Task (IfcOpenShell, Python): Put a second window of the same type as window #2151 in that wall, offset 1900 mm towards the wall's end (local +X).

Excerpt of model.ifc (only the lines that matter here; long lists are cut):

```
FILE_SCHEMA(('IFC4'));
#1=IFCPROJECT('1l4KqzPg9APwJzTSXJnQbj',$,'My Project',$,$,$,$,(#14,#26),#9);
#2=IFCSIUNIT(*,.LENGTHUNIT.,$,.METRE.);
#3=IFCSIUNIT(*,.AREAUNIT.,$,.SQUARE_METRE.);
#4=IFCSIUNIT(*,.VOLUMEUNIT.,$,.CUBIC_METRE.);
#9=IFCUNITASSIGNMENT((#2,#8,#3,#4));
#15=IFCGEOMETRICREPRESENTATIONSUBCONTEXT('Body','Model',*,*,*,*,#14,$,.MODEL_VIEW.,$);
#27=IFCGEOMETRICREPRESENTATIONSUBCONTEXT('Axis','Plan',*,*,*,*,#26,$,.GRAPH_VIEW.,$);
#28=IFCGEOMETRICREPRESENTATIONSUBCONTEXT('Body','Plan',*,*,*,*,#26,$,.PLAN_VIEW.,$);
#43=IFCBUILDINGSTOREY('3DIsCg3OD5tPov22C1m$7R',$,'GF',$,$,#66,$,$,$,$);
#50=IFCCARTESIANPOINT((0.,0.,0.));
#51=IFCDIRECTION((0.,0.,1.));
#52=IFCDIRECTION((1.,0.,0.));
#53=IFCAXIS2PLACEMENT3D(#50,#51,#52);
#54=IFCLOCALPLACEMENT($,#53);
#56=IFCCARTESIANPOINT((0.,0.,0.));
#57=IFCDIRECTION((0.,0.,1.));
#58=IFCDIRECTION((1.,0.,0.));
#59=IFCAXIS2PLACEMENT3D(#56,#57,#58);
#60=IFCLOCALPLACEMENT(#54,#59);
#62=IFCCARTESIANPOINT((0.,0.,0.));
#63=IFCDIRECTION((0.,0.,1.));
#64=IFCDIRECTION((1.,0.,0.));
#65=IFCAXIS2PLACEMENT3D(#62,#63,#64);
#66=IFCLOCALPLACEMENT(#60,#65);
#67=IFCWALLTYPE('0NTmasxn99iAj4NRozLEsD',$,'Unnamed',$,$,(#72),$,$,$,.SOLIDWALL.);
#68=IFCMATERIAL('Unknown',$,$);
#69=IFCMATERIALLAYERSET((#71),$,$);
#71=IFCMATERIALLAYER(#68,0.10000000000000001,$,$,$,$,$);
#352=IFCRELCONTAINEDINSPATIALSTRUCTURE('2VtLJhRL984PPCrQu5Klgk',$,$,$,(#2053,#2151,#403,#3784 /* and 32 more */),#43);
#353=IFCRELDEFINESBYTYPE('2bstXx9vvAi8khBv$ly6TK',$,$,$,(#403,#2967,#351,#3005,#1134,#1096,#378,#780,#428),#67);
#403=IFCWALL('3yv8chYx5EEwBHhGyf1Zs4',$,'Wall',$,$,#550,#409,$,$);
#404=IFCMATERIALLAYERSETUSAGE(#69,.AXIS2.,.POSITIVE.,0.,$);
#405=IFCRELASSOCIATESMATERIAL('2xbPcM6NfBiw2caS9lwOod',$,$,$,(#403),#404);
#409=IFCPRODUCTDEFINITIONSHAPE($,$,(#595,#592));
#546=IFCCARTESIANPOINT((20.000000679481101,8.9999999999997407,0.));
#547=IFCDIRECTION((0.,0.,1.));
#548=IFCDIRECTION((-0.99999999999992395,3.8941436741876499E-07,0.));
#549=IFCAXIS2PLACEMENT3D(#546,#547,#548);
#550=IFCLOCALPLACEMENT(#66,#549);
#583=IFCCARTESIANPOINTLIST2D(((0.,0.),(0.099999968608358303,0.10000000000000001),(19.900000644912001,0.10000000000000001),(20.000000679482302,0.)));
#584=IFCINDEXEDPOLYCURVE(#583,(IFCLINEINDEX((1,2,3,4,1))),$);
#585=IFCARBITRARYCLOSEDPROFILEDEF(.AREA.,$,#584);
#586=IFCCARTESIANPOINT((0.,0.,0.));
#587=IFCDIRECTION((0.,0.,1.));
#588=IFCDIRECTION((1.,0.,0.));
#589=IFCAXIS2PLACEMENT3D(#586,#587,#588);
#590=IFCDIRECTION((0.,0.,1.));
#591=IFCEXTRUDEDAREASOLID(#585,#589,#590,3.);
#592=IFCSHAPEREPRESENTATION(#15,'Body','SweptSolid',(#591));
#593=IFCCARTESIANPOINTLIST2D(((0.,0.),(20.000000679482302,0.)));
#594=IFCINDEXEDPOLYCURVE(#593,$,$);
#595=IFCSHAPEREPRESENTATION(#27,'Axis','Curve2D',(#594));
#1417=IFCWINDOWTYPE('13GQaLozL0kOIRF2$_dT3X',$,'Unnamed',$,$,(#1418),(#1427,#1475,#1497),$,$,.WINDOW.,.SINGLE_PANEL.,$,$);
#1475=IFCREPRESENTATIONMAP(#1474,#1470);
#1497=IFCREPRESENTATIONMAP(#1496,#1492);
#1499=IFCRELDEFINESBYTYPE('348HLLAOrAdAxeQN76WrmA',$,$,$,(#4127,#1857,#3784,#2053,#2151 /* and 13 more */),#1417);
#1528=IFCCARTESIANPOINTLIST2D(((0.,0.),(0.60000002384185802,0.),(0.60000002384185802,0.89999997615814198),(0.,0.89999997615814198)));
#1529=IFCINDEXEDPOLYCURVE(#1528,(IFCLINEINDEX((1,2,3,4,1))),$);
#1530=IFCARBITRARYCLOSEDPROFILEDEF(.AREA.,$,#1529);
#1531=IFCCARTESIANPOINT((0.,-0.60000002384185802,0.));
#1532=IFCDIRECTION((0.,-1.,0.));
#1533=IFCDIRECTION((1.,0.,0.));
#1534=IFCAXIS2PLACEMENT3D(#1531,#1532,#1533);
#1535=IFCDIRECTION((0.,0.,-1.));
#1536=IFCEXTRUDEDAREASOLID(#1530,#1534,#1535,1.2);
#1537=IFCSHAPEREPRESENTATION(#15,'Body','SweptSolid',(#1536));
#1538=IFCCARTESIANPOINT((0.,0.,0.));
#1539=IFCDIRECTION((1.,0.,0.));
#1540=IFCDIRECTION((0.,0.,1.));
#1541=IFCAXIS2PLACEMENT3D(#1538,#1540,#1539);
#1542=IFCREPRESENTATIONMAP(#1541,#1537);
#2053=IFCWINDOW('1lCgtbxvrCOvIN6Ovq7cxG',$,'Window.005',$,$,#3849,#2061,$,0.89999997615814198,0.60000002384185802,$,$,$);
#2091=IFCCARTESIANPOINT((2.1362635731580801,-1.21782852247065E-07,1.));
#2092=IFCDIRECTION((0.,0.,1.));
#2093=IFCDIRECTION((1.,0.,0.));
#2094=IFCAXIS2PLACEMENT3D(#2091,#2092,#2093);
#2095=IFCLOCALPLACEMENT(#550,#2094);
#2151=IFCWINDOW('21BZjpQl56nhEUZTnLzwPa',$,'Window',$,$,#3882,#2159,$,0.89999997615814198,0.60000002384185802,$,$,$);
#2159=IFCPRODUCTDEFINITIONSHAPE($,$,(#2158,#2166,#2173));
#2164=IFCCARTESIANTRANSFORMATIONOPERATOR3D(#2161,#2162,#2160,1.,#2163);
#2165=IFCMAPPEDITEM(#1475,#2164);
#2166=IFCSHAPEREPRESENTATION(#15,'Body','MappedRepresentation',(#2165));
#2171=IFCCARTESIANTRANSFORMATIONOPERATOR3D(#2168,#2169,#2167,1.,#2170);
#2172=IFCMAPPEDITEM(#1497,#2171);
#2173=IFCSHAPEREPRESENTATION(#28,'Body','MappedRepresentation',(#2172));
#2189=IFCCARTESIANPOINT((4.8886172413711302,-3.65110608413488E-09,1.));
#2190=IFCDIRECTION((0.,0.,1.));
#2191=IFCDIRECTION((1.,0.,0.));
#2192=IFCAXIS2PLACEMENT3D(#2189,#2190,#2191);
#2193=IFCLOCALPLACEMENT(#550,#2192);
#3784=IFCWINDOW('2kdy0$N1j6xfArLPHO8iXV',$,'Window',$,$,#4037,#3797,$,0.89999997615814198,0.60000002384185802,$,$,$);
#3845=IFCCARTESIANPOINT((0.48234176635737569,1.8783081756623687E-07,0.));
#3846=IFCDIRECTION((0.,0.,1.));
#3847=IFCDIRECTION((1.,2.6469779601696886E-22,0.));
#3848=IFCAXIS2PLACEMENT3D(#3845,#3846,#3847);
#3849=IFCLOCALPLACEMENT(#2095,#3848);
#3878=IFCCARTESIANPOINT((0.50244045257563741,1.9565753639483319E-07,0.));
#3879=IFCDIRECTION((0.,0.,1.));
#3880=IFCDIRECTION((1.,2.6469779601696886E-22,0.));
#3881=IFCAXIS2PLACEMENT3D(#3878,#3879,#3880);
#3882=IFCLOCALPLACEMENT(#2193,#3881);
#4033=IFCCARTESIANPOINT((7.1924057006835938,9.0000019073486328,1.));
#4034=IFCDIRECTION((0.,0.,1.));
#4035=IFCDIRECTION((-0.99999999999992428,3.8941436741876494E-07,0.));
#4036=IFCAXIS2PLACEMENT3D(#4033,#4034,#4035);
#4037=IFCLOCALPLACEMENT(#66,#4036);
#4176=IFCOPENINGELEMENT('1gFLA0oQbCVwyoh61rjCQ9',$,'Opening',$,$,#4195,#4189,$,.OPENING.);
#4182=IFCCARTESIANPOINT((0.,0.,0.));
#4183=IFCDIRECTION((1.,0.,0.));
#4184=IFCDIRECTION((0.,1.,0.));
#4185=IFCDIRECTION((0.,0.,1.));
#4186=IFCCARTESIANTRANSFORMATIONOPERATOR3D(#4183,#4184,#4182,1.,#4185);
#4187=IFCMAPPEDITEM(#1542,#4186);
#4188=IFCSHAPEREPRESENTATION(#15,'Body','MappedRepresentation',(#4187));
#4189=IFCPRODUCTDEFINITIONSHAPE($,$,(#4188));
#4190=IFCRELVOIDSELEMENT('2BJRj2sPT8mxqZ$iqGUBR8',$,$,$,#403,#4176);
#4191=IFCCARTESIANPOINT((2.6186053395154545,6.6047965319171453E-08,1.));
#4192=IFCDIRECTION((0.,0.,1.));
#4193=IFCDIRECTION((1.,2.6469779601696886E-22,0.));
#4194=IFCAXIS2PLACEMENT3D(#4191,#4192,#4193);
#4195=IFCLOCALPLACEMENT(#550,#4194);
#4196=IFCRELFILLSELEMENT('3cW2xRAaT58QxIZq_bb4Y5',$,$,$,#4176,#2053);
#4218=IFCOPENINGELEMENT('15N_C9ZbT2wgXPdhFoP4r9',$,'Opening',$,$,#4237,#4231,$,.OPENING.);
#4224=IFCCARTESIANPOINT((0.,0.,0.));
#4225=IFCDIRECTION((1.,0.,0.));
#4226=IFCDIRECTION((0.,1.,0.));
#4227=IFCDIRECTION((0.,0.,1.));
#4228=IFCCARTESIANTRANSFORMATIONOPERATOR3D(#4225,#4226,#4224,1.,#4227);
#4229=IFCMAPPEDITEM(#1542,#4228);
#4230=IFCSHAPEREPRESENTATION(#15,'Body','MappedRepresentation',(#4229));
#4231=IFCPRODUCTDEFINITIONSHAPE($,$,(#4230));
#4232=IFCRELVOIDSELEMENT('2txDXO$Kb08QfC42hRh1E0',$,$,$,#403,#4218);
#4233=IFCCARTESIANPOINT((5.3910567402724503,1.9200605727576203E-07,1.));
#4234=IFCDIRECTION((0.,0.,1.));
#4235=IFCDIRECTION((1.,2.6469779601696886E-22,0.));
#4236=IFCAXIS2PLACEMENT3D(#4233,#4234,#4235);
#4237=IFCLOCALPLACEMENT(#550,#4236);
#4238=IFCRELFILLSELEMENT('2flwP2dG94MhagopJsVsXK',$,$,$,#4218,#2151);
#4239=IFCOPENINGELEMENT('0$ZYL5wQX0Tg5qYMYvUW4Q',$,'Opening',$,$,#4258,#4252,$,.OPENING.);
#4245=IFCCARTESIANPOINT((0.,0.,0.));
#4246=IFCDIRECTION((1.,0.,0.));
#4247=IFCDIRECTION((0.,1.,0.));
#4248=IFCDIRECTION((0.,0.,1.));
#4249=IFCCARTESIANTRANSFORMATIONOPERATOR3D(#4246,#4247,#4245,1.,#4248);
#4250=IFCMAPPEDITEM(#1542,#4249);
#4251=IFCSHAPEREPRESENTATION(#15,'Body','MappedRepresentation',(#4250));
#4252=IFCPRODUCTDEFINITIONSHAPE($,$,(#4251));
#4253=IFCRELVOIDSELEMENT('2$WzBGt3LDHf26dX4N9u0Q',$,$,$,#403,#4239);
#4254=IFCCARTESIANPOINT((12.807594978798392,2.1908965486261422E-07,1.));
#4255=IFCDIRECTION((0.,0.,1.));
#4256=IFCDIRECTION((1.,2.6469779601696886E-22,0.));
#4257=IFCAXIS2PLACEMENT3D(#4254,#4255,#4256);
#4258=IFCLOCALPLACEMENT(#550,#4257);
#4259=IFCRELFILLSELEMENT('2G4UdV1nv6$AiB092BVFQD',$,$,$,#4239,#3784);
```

```python
import ifcopenshell
import ifcopenshell.api.feature
import ifcopenshell.api.geometry
import ifcopenshell.api.root
import ifcopenshell.geom
import ifcopenshell.util.element
import ifcopenshell.util.placement
import ifcopenshell.util.shape

model = ifcopenshell.open("model.ifc")
settings = ifcopenshell.geom.settings()


def volume(element):
    """Net volume in cubic metres, openings subtracted."""
    shape = ifcopenshell.geom.create_shape(settings, element)
    return ifcopenshell.util.shape.get_volume(shape.geometry)


window = model.by_guid("21BZjpQl56nhEUZTnLzwPa")
opening = window.FillsVoids[0].RelatingOpeningElement
wall = opening.VoidsElements[0].RelatingBuildingElement
before = volume(wall)
shift = ifcopenshell.util.placement.get_local_placement(wall.ObjectPlacement)[:3, 0] * 1.9

# copy_class copies the void relationship, type, container and properties, but no geometry.
new_opening = ifcopenshell.api.root.copy_class(model, product=opening)
new_opening.Representation = ifcopenshell.util.element.copy_deep(
    model, opening.Representation, exclude=["IfcGeometricRepresentationContext", "IfcRepresentationMap"]
)
new_window = ifcopenshell.api.root.copy_class(model, product=window)
new_window.Representation = ifcopenshell.util.element.copy_deep(
    model, window.Representation, exclude=["IfcGeometricRepresentationContext", "IfcRepresentationMap"]
)
ifcopenshell.api.feature.add_filling(model, opening=new_opening, element=new_window)

for old, new in ((opening, new_opening), (window, new_window)):
    matrix = ifcopenshell.util.placement.get_local_placement(old.ObjectPlacement)
    matrix[:3, 3] += shift
    ifcopenshell.api.geometry.edit_object_placement(model, product=new, matrix=matrix, is_si=False)

after = volume(wall)

print(f"wall volume {before:.3f} -> {after:.3f} m3")

model.write("model_v2.ifc")
```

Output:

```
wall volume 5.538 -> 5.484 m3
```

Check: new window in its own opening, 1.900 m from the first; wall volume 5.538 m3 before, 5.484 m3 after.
